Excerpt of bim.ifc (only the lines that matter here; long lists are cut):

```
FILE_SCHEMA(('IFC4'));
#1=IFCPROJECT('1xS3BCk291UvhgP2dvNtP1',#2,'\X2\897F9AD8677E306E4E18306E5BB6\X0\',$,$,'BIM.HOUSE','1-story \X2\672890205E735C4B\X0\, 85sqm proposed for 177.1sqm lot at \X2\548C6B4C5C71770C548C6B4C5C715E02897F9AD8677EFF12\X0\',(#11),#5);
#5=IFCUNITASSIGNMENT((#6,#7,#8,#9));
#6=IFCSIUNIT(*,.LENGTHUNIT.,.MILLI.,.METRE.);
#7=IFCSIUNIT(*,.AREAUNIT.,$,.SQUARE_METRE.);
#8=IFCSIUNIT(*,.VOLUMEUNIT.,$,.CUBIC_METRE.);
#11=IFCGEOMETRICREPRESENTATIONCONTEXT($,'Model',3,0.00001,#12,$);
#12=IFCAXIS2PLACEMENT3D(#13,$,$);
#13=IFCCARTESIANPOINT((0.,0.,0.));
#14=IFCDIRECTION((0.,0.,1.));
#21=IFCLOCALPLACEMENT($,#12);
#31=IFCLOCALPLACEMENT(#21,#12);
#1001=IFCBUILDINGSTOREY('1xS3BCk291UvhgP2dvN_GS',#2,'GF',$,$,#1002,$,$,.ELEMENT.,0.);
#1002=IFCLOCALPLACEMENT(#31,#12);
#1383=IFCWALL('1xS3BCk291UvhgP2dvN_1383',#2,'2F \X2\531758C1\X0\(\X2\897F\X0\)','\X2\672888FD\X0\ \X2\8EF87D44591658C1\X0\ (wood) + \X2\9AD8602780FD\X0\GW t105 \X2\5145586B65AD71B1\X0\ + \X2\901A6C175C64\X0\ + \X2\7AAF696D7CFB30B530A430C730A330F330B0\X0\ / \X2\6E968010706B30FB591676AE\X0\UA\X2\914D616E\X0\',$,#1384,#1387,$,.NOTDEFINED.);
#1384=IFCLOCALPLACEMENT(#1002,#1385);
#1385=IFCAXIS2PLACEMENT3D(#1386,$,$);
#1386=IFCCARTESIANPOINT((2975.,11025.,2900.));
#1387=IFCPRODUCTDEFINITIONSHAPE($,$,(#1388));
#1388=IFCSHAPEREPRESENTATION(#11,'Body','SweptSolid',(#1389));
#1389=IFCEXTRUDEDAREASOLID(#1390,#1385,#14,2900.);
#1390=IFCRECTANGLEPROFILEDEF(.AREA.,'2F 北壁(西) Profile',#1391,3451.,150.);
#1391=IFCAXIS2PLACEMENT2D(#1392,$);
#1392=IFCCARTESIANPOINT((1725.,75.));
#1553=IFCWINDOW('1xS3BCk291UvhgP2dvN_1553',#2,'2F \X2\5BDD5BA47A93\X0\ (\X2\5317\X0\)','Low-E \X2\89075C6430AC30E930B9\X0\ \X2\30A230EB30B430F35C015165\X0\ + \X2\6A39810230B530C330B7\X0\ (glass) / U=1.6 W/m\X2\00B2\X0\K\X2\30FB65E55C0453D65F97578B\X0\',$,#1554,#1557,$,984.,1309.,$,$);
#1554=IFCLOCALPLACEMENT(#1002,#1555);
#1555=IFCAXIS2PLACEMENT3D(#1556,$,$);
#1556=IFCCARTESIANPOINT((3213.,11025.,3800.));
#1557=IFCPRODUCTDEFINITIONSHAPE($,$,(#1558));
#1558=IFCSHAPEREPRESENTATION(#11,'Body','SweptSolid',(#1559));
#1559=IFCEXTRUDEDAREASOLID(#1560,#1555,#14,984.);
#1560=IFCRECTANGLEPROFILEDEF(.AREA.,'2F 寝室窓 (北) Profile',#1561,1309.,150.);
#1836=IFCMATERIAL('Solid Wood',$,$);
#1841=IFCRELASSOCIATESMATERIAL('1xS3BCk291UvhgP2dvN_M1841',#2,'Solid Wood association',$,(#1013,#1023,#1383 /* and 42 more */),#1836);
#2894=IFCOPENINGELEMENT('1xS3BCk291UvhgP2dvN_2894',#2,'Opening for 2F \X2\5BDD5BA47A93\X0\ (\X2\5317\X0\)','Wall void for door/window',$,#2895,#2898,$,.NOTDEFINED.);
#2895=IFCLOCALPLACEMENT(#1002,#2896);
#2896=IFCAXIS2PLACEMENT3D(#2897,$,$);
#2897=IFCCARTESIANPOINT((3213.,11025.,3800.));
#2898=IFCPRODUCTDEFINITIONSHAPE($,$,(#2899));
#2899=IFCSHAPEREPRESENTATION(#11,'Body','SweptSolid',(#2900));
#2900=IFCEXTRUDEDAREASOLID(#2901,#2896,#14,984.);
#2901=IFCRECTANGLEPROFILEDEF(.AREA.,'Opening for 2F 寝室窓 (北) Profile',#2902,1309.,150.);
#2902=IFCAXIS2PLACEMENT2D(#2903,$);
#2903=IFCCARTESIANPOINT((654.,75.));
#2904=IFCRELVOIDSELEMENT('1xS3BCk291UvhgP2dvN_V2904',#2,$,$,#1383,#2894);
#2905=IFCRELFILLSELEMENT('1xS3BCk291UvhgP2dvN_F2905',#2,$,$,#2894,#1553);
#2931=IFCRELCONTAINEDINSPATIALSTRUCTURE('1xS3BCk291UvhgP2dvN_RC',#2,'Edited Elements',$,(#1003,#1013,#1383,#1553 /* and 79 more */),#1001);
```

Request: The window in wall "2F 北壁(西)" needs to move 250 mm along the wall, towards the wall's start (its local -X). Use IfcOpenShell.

```python
import ifcopenshell
import ifcopenshell.api.geometry
import ifcopenshell.util.placement

model = ifcopenshell.open("bim.ifc")

window = model.by_guid("1xS3BCk291UvhgP2dvN_1553")
opening = window.FillsVoids[0].RelatingOpeningElement
wall = opening.VoidsElements[0].RelatingBuildingElement

wall_matrix = ifcopenshell.util.placement.get_local_placement(wall.ObjectPlacement)
shift = wall_matrix[:3, 0] * -250.0
before = ifcopenshell.util.placement.get_local_placement(window.ObjectPlacement)[:3, 3].copy()

# The window is not placed relative to its opening, so move both.
for product in (opening, window):
    matrix = ifcopenshell.util.placement.get_local_placement(product.ObjectPlacement)
    matrix[:3, 3] += shift
    ifcopenshell.api.geometry.edit_object_placement(model, product=product, matrix=matrix, is_si=False)

after = ifcopenshell.util.placement.get_local_placement(window.ObjectPlacement)[:3, 3]
print("window moved by", (after - before).round(3) + 0.0)

model.write("bim_updated.ifc")
```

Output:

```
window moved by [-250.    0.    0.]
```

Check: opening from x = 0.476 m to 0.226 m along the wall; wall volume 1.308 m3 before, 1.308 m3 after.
